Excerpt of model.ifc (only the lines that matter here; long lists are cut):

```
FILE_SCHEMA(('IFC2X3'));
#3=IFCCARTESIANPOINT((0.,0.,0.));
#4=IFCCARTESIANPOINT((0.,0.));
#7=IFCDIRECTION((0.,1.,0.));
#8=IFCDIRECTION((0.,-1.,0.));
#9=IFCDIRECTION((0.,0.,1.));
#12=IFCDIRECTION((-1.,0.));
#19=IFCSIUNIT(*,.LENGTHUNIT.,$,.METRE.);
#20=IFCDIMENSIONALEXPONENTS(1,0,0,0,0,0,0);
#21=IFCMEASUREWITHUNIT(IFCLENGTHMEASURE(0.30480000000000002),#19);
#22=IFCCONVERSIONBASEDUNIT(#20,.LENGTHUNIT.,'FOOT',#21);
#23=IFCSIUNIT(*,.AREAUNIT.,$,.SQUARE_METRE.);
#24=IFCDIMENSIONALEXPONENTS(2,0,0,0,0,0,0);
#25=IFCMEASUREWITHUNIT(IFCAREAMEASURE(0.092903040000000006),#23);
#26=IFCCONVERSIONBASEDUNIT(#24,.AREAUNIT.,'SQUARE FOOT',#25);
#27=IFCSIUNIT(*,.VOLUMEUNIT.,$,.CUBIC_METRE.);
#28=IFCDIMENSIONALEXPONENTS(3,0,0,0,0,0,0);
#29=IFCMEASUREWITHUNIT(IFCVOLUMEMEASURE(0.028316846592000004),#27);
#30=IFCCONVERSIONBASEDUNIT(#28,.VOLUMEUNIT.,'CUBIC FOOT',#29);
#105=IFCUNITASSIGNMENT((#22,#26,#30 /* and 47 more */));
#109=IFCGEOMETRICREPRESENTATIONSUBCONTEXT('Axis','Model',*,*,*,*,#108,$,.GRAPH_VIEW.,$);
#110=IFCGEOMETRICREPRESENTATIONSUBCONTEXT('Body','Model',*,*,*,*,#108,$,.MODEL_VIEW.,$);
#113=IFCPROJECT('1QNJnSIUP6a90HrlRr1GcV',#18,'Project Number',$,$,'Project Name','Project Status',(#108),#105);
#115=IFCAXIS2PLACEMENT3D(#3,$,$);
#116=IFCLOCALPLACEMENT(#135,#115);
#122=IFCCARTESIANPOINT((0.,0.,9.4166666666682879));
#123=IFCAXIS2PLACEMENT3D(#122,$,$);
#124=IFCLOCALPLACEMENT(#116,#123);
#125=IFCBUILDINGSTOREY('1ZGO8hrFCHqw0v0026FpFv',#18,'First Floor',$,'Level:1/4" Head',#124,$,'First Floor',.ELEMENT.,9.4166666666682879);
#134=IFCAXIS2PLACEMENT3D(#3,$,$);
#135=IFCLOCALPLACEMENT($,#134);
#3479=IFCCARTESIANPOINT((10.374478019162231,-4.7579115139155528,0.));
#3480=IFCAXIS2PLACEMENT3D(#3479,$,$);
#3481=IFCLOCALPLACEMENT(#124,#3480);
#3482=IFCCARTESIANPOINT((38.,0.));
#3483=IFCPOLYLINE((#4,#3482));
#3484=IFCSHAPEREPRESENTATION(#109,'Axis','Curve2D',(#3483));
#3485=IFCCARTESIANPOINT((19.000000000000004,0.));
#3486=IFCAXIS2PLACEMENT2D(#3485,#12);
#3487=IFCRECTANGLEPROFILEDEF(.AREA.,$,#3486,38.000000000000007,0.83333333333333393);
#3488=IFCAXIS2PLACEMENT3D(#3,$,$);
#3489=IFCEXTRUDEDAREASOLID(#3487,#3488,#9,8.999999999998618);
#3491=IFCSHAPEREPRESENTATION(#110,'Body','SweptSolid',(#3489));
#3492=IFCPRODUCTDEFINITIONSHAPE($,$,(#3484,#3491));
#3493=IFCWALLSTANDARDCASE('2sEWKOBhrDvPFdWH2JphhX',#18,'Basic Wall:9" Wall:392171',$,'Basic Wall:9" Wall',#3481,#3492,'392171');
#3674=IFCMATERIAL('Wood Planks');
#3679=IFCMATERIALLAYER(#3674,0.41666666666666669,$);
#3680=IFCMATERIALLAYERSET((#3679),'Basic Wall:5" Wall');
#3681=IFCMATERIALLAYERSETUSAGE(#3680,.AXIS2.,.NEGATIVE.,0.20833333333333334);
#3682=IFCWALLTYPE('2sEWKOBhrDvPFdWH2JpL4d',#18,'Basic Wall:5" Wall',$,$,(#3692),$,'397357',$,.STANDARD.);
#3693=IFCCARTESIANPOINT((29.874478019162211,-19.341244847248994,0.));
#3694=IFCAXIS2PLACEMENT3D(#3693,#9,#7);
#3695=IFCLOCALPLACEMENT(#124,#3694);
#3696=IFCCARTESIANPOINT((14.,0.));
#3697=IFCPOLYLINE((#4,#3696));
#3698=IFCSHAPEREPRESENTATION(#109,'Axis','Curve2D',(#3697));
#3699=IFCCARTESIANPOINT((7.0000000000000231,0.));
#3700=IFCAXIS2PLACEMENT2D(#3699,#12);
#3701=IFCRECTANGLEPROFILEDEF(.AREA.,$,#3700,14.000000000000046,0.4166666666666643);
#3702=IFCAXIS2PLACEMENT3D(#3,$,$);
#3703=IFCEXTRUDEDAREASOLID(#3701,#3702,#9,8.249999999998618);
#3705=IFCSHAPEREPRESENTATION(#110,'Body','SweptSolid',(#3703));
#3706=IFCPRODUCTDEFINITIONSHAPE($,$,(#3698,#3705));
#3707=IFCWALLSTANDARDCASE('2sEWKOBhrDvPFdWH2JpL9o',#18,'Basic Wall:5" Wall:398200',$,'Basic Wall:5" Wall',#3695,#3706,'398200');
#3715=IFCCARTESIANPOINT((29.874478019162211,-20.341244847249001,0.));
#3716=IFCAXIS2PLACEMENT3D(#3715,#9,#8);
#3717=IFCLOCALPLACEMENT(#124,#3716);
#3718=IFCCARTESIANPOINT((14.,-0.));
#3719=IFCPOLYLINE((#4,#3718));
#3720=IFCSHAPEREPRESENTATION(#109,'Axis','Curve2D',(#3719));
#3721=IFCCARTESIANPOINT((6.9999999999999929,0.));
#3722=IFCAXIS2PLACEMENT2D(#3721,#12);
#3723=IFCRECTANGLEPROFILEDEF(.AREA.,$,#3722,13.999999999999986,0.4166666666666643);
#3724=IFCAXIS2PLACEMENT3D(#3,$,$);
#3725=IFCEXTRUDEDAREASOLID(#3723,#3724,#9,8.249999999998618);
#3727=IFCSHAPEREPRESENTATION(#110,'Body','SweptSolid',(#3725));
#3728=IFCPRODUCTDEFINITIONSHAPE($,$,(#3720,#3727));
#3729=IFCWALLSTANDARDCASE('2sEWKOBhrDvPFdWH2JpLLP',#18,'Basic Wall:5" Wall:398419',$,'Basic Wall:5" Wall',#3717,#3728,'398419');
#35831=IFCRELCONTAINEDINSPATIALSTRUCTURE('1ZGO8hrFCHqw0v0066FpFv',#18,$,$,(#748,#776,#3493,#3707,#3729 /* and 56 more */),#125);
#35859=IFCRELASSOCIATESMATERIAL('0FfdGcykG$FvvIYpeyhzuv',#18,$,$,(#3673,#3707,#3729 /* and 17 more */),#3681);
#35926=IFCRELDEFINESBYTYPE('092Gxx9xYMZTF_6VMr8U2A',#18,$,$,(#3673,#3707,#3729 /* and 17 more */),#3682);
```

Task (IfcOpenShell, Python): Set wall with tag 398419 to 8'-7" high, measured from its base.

```python
import ifcopenshell
import ifcopenshell.geom
import ifcopenshell.util.representation
import ifcopenshell.util.shape
import ifcopenshell.util.unit

model = ifcopenshell.open("model.ifc")
unit_scale = ifcopenshell.util.unit.calculate_unit_scale(model)
settings = ifcopenshell.geom.settings()


def volume(element):
    """Net volume in cubic metres, openings subtracted."""
    shape = ifcopenshell.geom.create_shape(settings, element)
    return ifcopenshell.util.shape.get_volume(shape.geometry)


wall = model.by_id(3729)
before = volume(wall)

body = ifcopenshell.util.representation.get_representation(wall, "Model", "Body")
solid = body.Items[0]
old_height = solid.Depth
solid.Depth = 103 * 0.0254 / unit_scale
after = volume(wall)

print(f"height {old_height:g} -> {solid.Depth:g}, volume {before:.3f} -> {after:.3f} m3")

model.write("model_updated.ifc")
```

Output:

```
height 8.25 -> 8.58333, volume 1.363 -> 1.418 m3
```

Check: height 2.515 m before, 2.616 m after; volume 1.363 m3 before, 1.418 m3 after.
